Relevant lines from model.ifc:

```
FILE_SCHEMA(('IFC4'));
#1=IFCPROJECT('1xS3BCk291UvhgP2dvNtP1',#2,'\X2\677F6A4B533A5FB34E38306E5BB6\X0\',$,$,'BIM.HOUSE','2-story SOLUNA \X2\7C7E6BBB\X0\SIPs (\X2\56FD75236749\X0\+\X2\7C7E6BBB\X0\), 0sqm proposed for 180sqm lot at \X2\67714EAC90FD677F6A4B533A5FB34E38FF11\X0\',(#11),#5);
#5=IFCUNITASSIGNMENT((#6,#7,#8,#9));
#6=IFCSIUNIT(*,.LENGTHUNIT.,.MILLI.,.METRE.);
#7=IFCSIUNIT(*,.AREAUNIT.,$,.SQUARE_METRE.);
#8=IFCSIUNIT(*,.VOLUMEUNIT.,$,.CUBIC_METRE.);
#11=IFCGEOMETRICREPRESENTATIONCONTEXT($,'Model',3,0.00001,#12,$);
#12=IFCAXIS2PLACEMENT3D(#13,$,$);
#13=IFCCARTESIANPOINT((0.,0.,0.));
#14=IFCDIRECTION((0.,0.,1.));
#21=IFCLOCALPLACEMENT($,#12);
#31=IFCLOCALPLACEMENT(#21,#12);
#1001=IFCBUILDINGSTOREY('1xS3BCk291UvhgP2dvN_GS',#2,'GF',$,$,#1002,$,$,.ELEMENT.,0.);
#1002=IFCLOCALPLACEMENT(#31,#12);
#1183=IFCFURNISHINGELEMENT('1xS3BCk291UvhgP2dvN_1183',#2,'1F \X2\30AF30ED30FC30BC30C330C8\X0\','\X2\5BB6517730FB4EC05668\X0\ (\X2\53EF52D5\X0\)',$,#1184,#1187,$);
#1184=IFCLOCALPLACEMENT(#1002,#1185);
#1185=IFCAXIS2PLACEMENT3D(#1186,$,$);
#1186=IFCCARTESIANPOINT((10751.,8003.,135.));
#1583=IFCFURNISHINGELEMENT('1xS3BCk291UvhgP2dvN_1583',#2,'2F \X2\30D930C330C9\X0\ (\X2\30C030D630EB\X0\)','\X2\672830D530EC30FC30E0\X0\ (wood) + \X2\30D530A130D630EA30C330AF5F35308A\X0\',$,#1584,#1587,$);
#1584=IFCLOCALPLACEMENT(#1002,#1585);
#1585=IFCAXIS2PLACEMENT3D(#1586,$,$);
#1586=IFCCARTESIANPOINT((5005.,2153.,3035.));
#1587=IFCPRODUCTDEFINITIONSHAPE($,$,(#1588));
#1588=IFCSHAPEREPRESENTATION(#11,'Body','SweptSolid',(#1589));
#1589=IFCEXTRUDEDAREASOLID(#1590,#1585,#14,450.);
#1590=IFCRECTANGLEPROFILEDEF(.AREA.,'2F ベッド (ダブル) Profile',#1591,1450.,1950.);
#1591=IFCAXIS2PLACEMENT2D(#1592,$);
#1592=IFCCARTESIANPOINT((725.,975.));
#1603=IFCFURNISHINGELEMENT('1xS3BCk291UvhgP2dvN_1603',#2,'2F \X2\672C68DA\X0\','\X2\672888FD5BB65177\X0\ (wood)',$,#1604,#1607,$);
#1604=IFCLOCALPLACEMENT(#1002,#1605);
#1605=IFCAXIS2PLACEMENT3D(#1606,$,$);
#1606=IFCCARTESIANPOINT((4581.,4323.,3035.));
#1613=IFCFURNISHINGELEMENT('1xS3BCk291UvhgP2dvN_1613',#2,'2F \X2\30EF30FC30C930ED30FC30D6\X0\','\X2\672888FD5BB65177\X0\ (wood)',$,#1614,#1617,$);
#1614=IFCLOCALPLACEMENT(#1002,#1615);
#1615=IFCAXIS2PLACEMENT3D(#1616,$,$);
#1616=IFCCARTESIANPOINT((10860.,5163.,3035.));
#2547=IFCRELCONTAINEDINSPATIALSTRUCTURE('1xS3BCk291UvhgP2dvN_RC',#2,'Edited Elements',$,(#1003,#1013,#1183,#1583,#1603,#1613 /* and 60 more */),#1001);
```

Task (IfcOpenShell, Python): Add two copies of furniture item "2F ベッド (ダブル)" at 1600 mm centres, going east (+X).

```python
import numpy as np
import ifcopenshell
import ifcopenshell.api.geometry
import ifcopenshell.api.root
import ifcopenshell.util.element
import ifcopenshell.util.placement

model = ifcopenshell.open("model.ifc")


def reuse_history(source, copy):
    """copy_class also copies each property set's owner history, people and application; keep the originals."""
    for rel in copy.IsDefinedBy:
        if rel.is_a("IfcRelDefinesByProperties") and (history := rel.RelatingPropertyDefinition.OwnerHistory):
            rel.RelatingPropertyDefinition.OwnerHistory = source.OwnerHistory
            ifcopenshell.util.element.remove_deep2(model, history)


source = model.by_id(1583)
base = ifcopenshell.util.placement.get_local_placement(source.ObjectPlacement)
step = np.array([1.0, 0.0, 0.0]) * 1600.0

for i in range(1, 3):
    copy = ifcopenshell.api.root.copy_class(model, product=source)
    copy.Representation = ifcopenshell.util.element.copy_deep(
        model, source.Representation, exclude=["IfcGeometricRepresentationContext", "IfcRepresentationMap"]
    )
    reuse_history(source, copy)
    matrix = base.copy()
    matrix[:3, 3] += i * step
    print("added at", matrix[:3, 3].round(3) + 0.0)
    ifcopenshell.api.geometry.edit_object_placement(model, product=copy, matrix=matrix, is_si=False)

model.write("model_v2.ifc")
```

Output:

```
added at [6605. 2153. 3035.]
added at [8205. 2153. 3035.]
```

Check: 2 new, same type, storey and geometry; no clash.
